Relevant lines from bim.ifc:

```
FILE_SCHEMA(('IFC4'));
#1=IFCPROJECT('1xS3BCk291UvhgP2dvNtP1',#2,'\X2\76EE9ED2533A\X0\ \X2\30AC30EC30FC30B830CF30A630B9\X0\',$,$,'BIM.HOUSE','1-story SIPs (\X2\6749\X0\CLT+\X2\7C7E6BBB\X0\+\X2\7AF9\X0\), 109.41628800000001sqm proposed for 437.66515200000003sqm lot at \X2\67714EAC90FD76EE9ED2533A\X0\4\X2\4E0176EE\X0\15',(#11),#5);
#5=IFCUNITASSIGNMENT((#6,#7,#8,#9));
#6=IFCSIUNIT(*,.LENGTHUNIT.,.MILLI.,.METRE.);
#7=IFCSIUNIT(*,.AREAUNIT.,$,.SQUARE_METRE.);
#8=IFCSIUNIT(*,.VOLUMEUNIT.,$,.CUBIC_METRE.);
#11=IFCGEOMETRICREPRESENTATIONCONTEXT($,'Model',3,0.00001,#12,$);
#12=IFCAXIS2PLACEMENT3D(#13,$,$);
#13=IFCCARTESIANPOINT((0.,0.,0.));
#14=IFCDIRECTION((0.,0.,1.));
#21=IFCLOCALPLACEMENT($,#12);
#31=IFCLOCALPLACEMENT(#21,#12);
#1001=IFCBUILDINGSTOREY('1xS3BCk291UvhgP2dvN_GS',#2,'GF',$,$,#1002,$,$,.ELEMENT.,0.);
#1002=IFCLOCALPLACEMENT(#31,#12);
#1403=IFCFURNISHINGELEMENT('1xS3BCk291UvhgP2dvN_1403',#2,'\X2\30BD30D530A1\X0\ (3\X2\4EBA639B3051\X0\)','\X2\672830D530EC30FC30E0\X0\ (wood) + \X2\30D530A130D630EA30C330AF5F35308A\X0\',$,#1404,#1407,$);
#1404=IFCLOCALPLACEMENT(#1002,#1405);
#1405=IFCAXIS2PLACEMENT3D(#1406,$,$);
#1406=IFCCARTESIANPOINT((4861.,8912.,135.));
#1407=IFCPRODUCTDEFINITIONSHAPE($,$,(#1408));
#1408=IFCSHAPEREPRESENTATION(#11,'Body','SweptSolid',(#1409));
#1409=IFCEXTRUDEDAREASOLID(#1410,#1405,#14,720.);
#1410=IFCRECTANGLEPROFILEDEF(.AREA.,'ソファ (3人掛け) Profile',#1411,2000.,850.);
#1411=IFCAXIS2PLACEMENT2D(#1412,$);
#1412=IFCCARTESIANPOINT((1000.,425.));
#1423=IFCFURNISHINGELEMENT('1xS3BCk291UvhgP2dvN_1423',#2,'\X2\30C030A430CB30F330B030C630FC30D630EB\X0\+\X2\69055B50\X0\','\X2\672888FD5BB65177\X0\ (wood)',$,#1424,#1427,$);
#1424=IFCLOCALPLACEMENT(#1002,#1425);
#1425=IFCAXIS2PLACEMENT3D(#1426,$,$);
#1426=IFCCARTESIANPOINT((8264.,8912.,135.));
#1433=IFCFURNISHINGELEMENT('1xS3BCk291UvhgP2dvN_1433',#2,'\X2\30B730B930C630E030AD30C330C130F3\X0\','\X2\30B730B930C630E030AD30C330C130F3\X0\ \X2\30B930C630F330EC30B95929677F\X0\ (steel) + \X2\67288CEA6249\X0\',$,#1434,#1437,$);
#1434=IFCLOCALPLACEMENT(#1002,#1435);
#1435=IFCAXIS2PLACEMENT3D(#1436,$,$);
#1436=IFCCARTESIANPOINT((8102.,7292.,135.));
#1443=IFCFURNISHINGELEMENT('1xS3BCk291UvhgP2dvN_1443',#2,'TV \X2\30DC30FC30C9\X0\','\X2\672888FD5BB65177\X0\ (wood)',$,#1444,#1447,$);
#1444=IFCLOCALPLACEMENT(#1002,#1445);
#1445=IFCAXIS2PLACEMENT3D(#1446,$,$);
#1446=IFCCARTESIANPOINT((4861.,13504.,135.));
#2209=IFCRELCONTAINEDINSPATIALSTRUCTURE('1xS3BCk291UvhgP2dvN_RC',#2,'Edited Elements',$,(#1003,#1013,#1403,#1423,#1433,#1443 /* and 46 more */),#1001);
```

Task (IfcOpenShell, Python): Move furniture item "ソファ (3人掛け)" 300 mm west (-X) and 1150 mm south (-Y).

```python
import ifcopenshell
import ifcopenshell.api.geometry
import ifcopenshell.util.placement
import ifcopenshell.util.unit

model = ifcopenshell.open("bim.ifc")
unit_scale = ifcopenshell.util.unit.calculate_unit_scale(model)

item = model.by_id(1403)
matrix = ifcopenshell.util.placement.get_local_placement(item.ObjectPlacement)
matrix[0, 3] -= 0.3 / unit_scale
matrix[1, 3] -= 1.15 / unit_scale
ifcopenshell.api.geometry.edit_object_placement(model, product=item, matrix=matrix, is_si=False)

print(ifcopenshell.util.placement.get_local_placement(item.ObjectPlacement).round(3) + 0.0)

model.write("bim_updated.ifc")
```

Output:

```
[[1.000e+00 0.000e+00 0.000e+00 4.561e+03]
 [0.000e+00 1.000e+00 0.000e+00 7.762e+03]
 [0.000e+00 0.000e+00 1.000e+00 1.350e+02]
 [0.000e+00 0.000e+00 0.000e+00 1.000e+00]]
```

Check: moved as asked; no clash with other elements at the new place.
